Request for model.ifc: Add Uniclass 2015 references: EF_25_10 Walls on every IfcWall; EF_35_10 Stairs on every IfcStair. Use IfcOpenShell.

First a look at what the model holds.

```python
import ifcopenshell

model = ifcopenshell.open("model.ifc")
print(model.schema)
print("classifications:", [c.Name for c in model.by_type("IfcClassification")])
for ifc_class in ("IfcDoor", "IfcRoof", "IfcStair", "IfcWall", "IfcWindow"):
    print(ifc_class, len(model.by_type(ifc_class)))
```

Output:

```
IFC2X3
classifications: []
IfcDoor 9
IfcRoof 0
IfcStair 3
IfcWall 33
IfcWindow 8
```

```python
import ifcopenshell
import ifcopenshell.api.classification

model = ifcopenshell.open("model.ifc")

# IFC2X3 requires Source and Edition and has no link from the project to the system.
system = model.create_entity("IfcClassification", Source="NBS", Edition="2015", Name="Uniclass 2015")

codes = {
    "IfcWall": ("EF_25_10", "Walls"),
    "IfcStair": ("EF_35_10", "Stairs"),
}
for ifc_class, (code, name) in codes.items():
    products = model.by_type(ifc_class)
    ifcopenshell.api.classification.add_reference(
        model, products=products, classification=system, identification=code, name=name
    )
    print(code, len(products))

model.write("model_edited.ifc")
```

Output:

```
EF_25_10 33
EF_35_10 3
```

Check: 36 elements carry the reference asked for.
